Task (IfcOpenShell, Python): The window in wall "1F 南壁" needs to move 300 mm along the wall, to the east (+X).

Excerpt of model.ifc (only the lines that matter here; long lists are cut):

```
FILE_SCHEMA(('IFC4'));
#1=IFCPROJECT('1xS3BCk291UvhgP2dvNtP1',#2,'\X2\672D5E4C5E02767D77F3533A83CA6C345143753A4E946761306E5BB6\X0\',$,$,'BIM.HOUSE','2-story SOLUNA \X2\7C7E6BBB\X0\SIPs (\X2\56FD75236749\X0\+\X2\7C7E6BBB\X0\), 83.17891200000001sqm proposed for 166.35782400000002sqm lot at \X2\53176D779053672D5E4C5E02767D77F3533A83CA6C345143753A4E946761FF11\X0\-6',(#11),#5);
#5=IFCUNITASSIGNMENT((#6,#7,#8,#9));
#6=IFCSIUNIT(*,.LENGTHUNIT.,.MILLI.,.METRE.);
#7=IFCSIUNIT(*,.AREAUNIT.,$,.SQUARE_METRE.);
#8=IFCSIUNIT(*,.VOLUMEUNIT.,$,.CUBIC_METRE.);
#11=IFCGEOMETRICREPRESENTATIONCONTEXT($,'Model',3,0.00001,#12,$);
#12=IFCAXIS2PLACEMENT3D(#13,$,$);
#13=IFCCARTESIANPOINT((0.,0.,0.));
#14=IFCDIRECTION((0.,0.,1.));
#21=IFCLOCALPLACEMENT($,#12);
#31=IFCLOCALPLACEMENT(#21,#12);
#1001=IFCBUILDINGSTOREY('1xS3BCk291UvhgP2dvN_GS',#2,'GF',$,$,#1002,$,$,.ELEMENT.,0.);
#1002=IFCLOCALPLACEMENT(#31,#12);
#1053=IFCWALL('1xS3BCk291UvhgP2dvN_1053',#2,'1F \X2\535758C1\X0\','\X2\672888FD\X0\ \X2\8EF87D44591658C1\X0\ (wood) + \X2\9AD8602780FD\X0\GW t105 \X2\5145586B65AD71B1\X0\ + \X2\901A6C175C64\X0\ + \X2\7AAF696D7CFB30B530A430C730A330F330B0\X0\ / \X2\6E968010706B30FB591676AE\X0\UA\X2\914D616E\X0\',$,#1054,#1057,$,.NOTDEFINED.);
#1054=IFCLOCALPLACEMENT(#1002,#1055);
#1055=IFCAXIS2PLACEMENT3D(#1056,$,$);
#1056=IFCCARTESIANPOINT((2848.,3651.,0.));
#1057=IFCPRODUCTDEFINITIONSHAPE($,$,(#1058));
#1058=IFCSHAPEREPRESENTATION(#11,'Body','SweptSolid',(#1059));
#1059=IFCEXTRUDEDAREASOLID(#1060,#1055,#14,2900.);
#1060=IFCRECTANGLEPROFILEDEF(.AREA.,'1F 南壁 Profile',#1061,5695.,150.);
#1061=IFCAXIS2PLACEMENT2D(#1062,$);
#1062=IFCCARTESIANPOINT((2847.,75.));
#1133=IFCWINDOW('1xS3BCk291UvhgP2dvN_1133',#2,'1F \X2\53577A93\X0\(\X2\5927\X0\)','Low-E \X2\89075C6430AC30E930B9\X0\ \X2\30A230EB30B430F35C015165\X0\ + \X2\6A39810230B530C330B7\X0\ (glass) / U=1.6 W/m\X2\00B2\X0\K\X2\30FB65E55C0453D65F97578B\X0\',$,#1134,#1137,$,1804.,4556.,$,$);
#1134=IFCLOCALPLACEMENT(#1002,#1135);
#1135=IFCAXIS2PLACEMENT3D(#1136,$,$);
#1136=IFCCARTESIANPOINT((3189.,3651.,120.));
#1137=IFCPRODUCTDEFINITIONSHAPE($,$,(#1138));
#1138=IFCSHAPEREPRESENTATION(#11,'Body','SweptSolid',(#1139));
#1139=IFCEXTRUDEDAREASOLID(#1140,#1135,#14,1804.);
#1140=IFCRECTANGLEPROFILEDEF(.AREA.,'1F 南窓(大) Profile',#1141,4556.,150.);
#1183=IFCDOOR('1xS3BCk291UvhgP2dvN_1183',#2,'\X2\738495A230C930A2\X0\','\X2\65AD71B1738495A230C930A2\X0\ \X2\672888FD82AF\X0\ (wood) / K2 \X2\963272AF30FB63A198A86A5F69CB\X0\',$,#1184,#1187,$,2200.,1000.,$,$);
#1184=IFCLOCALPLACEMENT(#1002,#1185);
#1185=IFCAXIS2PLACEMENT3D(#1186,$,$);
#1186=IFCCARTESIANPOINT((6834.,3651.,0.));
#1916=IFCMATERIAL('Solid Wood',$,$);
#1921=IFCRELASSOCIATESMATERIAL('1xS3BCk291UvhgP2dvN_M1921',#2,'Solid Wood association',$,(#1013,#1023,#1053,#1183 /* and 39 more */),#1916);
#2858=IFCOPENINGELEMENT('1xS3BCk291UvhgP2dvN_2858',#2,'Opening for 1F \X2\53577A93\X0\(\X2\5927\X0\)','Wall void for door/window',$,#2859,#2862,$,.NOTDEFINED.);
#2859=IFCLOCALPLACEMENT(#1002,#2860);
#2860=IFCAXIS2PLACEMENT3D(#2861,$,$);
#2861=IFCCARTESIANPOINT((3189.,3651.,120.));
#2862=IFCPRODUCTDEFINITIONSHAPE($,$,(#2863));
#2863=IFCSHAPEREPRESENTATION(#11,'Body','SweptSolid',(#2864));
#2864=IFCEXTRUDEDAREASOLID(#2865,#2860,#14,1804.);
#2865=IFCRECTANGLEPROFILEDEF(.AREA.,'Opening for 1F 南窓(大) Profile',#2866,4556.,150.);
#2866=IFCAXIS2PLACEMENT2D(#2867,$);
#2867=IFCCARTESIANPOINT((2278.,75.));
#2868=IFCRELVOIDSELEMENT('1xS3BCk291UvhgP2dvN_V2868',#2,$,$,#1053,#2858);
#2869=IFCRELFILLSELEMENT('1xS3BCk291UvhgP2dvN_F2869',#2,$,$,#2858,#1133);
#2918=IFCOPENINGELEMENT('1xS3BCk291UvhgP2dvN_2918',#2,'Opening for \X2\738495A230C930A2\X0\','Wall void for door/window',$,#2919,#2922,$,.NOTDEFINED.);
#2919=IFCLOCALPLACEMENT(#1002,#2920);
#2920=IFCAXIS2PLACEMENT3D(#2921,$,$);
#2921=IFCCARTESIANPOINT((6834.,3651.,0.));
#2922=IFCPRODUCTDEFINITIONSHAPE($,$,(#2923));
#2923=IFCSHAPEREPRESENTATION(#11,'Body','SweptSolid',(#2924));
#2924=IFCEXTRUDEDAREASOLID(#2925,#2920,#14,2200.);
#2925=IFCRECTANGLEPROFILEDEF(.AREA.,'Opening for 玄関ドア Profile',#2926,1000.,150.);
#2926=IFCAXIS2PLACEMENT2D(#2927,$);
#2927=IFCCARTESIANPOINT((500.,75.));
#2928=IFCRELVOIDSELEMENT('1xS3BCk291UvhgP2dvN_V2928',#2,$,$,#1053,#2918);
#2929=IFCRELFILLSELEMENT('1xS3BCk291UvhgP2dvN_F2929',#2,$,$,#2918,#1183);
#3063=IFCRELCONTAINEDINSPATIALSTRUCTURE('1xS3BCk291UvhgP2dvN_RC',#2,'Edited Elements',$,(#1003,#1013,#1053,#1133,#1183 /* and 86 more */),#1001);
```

```python
import ifcopenshell
import ifcopenshell.api.geometry
import ifcopenshell.util.placement

model = ifcopenshell.open("model.ifc")

window = model.by_guid("1xS3BCk291UvhgP2dvN_1133")
opening = window.FillsVoids[0].RelatingOpeningElement
wall = opening.VoidsElements[0].RelatingBuildingElement

wall_matrix = ifcopenshell.util.placement.get_local_placement(wall.ObjectPlacement)
shift = wall_matrix[:3, 0] * 300.0
before = ifcopenshell.util.placement.get_local_placement(window.ObjectPlacement)[:3, 3].copy()

# The window is not placed relative to its opening, so move both.
for product in (opening, window):
    matrix = ifcopenshell.util.placement.get_local_placement(product.ObjectPlacement)
    matrix[:3, 3] += shift
    ifcopenshell.api.geometry.edit_object_placement(model, product=product, matrix=matrix, is_si=False)

after = ifcopenshell.util.placement.get_local_placement(window.ObjectPlacement)[:3, 3]
print("window moved by", (after - before).round(3) + 0.0)

model.write("model_updated.ifc")
```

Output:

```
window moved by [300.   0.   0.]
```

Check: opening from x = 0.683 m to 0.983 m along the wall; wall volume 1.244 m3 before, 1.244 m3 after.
